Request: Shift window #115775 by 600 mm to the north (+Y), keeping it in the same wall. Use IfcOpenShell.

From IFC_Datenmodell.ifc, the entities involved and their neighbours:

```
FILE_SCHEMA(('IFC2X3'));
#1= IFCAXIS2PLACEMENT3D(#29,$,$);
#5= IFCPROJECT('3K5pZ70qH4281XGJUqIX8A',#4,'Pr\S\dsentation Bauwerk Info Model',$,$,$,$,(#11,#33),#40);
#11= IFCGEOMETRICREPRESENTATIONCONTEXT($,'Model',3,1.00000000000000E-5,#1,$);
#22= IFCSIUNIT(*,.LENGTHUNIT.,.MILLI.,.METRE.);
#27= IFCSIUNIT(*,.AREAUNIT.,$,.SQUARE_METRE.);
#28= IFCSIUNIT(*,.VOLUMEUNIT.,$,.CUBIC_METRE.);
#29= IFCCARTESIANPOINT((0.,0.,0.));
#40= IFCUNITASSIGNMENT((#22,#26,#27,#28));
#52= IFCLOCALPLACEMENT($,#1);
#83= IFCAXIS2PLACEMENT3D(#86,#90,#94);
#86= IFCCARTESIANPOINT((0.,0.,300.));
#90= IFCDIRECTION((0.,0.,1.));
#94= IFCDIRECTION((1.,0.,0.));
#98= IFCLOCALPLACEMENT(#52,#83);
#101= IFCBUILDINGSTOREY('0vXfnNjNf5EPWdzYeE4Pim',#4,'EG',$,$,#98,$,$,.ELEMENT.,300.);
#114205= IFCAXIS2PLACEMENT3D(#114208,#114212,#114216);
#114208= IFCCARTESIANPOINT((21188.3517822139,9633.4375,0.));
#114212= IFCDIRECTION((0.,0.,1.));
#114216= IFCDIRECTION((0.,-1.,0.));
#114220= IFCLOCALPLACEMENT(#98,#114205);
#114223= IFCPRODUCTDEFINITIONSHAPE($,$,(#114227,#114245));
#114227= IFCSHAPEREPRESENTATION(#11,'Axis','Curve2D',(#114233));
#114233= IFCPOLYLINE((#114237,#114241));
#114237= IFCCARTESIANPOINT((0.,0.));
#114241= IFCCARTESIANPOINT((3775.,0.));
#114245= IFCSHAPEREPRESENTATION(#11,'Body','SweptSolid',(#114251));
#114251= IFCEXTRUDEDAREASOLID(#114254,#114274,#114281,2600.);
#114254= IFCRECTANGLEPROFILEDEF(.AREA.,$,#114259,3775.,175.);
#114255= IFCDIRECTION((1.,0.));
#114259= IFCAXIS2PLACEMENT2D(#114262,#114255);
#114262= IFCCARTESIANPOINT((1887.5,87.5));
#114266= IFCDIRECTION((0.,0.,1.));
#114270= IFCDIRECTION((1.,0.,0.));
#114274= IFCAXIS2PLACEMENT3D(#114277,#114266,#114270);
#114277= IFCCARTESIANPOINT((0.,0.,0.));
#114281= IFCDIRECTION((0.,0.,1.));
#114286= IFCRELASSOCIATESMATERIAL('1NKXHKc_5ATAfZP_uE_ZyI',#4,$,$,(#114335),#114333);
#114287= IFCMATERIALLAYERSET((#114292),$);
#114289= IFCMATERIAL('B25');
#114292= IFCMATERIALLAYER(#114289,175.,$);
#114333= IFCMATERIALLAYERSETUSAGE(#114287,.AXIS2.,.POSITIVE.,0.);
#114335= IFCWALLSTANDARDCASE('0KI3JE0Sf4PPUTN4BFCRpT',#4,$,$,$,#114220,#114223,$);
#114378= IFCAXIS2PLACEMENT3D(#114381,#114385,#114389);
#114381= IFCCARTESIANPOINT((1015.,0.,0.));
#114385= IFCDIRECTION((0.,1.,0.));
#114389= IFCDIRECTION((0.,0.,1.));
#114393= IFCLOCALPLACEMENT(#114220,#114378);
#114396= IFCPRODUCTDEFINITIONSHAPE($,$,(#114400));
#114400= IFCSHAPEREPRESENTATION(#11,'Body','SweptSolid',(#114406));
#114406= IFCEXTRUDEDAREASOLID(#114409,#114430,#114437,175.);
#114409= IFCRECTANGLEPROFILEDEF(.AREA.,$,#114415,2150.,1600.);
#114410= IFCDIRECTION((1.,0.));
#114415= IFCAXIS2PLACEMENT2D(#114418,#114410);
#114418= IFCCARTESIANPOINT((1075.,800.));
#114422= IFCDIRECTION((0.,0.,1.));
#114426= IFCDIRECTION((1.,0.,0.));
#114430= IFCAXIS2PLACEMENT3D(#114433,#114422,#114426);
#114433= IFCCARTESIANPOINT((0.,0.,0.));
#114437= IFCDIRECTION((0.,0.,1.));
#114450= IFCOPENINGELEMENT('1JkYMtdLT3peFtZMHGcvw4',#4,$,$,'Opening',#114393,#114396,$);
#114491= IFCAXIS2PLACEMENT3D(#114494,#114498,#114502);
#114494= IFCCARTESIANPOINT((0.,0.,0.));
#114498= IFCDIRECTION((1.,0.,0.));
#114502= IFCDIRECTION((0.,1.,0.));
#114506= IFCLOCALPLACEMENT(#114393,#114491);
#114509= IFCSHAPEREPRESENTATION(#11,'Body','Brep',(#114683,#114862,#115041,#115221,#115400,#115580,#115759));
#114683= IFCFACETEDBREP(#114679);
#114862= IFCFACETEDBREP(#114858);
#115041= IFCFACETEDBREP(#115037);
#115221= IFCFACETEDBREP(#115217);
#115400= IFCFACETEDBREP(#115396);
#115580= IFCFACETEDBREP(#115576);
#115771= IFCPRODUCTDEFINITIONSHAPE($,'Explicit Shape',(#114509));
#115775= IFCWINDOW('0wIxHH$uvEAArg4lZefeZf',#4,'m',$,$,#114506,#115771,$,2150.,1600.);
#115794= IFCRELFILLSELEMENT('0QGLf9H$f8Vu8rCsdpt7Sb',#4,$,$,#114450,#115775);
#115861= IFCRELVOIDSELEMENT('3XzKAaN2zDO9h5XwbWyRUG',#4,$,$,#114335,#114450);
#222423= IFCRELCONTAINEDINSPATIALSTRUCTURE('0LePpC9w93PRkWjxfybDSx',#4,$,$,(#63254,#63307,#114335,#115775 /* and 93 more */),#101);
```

```python
import ifcopenshell
import ifcopenshell.api.geometry
import ifcopenshell.util.placement
import ifcopenshell.util.unit

model = ifcopenshell.open("IFC_Datenmodell.ifc")
unit_scale = ifcopenshell.util.unit.calculate_unit_scale(model)

window = model.by_id(115775)
opening = window.FillsVoids[0].RelatingOpeningElement
wall = opening.VoidsElements[0].RelatingBuildingElement

wall_matrix = ifcopenshell.util.placement.get_local_placement(wall.ObjectPlacement)
shift = wall_matrix[:3, 0] * -0.6 / unit_scale
before = ifcopenshell.util.placement.get_local_placement(window.ObjectPlacement)[:3, 3].copy()

# The window is placed relative to its opening, so it follows when the opening moves.
matrix = ifcopenshell.util.placement.get_local_placement(opening.ObjectPlacement)
matrix[:3, 3] += shift
ifcopenshell.api.geometry.edit_object_placement(
    model, product=opening, matrix=matrix, is_si=False, should_transform_children=True
)

after = ifcopenshell.util.placement.get_local_placement(window.ObjectPlacement)[:3, 3]
print("window moved by", (after - before).round(3) + 0.0)

model.write("IFC_Datenmodell_rev.ifc")
```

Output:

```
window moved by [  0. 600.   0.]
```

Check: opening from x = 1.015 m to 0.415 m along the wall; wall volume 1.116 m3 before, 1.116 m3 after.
